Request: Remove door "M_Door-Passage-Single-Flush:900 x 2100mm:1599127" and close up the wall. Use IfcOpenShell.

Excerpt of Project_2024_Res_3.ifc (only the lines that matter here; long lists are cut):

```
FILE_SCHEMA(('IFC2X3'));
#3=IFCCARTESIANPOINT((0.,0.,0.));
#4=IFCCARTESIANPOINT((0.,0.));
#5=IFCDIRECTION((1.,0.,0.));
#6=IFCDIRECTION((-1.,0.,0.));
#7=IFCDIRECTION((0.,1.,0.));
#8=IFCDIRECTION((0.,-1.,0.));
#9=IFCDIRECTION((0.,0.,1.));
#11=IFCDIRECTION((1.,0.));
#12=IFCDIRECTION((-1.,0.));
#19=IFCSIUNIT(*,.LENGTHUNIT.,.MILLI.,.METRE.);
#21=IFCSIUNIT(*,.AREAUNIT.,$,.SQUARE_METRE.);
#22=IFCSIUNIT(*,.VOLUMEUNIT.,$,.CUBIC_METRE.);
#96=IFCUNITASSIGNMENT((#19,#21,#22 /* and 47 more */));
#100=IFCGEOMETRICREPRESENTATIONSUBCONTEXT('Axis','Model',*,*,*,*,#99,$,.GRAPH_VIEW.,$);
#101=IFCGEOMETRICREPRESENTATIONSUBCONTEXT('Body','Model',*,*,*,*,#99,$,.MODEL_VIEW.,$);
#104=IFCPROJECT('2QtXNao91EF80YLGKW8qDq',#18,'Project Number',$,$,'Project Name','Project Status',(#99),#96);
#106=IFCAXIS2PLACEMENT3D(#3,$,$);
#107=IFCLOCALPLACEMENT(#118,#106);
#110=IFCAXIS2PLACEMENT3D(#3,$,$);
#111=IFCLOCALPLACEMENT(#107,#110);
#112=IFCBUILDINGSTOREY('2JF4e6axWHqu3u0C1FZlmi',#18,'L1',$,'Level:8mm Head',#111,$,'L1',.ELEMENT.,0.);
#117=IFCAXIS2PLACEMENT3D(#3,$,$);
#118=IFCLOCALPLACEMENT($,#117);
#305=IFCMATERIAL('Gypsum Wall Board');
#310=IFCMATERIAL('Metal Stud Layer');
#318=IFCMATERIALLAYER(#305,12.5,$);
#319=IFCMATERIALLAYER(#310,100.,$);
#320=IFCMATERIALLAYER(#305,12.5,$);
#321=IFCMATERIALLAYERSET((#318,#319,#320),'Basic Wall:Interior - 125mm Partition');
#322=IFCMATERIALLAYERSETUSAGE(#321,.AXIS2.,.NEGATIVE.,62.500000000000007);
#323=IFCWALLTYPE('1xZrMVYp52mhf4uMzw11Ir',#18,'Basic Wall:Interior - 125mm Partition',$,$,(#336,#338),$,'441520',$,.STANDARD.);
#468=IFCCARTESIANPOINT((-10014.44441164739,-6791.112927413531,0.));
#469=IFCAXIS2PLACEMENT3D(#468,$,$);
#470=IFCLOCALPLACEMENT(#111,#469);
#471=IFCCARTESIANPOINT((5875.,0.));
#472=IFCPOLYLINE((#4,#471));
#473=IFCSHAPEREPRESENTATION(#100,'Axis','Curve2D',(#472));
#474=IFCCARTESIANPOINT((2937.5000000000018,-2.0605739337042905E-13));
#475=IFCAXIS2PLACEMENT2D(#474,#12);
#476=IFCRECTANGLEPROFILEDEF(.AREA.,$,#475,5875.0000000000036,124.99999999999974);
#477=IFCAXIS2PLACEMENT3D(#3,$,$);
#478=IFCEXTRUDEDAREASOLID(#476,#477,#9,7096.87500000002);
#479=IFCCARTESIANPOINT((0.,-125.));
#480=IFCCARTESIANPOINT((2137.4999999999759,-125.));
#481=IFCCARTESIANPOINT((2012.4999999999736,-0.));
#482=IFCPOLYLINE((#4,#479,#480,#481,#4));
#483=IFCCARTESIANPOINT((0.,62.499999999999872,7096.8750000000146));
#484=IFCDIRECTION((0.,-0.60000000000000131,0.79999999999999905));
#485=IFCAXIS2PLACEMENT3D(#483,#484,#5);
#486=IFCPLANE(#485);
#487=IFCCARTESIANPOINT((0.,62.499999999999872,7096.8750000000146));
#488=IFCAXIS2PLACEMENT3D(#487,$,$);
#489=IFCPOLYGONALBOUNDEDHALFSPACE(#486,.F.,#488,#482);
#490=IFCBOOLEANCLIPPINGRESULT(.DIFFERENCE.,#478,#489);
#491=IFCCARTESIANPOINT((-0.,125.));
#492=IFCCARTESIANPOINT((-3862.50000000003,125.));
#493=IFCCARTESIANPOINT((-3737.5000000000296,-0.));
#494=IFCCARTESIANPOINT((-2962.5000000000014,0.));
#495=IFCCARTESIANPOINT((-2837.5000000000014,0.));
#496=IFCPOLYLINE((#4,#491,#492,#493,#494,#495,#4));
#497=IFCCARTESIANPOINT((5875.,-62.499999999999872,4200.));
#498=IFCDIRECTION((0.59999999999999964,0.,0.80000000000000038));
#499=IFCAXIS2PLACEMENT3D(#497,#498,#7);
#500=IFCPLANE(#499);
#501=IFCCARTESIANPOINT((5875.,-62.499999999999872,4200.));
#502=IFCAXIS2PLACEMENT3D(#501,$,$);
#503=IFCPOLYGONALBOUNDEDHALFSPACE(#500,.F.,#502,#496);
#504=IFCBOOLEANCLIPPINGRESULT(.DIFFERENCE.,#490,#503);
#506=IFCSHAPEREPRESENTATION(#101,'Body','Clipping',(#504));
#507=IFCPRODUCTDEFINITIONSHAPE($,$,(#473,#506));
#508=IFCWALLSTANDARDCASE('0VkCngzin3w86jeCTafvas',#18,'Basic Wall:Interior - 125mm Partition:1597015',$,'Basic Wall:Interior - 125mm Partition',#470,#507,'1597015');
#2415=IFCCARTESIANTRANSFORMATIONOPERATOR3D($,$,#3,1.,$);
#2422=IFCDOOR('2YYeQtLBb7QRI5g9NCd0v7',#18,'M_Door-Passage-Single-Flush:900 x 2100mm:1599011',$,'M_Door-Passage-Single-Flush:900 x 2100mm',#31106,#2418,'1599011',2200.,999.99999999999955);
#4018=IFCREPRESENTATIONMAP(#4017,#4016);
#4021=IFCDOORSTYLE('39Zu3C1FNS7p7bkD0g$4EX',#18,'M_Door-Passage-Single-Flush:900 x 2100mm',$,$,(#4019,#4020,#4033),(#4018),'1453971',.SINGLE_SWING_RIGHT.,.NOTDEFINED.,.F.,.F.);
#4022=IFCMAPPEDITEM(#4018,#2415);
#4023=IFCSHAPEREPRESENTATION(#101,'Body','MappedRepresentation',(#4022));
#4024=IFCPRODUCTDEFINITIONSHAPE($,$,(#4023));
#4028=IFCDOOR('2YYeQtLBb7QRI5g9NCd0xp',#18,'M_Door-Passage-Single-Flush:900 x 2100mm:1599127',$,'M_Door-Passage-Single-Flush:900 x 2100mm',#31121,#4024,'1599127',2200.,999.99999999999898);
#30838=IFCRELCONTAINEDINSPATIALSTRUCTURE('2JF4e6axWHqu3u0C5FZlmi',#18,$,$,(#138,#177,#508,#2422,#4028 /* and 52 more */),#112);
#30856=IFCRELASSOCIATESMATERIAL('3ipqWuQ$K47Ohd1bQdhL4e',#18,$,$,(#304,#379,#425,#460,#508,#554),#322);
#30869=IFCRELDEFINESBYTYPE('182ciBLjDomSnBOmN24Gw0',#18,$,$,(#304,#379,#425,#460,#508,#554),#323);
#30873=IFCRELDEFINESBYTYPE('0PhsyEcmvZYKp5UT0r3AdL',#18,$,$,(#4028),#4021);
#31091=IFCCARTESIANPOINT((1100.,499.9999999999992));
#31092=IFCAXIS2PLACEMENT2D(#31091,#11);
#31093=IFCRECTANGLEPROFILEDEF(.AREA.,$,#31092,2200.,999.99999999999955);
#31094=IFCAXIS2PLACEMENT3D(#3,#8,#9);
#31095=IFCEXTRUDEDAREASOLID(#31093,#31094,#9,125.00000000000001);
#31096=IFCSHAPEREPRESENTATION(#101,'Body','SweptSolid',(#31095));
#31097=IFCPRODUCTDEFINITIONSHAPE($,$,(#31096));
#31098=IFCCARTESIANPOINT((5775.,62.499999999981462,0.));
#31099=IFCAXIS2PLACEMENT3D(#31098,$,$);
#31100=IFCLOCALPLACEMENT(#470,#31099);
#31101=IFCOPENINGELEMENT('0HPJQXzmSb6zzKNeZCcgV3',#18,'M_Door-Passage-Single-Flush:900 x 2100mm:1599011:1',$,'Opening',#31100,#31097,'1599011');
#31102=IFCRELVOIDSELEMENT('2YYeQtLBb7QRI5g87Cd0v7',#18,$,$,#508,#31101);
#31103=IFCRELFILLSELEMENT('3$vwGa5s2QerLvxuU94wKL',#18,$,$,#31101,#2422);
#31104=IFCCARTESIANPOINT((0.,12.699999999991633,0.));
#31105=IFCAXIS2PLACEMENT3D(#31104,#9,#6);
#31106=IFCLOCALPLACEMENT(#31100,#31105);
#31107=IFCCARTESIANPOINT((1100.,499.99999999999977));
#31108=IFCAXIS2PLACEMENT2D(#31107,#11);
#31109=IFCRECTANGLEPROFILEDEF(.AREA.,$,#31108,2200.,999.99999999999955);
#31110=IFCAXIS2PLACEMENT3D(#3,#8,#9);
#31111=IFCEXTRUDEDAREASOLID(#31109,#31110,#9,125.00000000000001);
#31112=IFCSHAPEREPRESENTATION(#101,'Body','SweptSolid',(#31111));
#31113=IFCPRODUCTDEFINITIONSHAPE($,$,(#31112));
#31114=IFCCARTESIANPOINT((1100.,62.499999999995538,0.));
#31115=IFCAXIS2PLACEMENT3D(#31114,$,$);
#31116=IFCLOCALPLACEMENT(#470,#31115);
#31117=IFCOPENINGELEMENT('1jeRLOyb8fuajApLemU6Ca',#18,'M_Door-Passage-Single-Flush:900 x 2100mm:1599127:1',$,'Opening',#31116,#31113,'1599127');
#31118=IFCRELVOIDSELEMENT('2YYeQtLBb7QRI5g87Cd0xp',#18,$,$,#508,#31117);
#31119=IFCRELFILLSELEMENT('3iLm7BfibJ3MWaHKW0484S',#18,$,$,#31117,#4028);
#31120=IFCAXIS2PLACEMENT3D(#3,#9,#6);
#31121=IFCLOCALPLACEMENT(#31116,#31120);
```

```python
import ifcopenshell
import ifcopenshell.api.feature
import ifcopenshell.api.root
import ifcopenshell.geom
import ifcopenshell.util.shape

model = ifcopenshell.open("Project_2024_Res_3.ifc")
settings = ifcopenshell.geom.settings()


def volume(element):
    """Net volume in cubic metres, openings subtracted."""
    shape = ifcopenshell.geom.create_shape(settings, element)
    return ifcopenshell.util.shape.get_volume(shape.geometry)


door = model.by_guid("2YYeQtLBb7QRI5g9NCd0xp")
opening = door.FillsVoids[0].RelatingOpeningElement
wall = opening.VoidsElements[0].RelatingBuildingElement
before = volume(wall)

ifcopenshell.api.root.remove_product(model, product=door)
ifcopenshell.api.feature.remove_feature(model, feature=opening)

after = volume(wall)

print(f"wall volume {before:.3f} -> {after:.3f} m3")

model.write("Project_2024_Res_3-out.ifc")
```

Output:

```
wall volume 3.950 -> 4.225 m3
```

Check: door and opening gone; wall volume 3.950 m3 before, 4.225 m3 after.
